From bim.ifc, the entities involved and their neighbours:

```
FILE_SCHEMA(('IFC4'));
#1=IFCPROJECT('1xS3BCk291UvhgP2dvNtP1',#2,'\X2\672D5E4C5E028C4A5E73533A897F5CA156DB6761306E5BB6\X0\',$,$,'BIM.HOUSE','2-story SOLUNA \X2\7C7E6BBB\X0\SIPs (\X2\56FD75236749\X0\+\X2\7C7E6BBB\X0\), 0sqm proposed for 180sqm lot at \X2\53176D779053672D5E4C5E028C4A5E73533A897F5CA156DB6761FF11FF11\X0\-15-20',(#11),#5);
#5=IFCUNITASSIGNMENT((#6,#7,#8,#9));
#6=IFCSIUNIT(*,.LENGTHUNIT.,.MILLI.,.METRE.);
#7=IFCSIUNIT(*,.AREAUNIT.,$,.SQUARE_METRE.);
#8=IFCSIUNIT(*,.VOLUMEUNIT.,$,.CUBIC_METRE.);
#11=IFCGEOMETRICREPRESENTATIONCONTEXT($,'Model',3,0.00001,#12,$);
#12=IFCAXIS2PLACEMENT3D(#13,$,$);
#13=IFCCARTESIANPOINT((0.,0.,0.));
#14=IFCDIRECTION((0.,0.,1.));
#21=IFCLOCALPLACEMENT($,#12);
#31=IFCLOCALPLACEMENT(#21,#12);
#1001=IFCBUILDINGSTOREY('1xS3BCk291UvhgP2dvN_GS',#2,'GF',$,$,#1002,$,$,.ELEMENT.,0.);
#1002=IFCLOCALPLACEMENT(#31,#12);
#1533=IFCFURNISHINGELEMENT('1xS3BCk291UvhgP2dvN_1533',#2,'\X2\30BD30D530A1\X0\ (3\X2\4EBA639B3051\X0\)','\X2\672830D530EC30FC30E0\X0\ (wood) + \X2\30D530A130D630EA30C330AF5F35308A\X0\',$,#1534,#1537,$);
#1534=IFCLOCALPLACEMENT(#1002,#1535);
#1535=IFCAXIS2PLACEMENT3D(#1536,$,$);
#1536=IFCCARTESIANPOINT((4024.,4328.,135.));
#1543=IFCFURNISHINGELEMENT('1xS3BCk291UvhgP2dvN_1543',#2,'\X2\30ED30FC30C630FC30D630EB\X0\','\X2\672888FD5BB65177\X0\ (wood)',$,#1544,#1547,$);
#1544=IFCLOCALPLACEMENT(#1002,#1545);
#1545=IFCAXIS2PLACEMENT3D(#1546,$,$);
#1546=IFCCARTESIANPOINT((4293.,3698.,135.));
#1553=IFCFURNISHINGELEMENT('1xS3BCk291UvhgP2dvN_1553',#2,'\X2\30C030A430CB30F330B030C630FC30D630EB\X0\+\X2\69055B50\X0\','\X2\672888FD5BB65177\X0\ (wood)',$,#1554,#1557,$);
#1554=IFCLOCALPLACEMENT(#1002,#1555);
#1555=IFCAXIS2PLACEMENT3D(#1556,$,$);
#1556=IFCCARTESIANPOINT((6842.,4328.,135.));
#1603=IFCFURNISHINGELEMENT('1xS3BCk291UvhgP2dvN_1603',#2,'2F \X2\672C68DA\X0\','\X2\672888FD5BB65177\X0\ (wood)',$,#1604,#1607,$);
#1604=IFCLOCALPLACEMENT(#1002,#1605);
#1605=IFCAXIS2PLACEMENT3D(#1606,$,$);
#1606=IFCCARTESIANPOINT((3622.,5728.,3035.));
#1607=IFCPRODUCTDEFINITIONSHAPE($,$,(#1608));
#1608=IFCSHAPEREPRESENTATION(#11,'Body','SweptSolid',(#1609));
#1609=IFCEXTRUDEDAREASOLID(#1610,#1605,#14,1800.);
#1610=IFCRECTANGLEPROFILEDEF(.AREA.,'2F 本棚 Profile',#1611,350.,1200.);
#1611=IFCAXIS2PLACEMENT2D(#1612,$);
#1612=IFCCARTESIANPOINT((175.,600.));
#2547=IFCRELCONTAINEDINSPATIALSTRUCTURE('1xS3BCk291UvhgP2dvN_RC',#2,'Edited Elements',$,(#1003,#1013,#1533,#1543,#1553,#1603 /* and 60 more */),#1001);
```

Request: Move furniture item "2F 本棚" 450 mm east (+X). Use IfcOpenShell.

```python
import ifcopenshell
import ifcopenshell.api.geometry
import ifcopenshell.util.placement

model = ifcopenshell.open("bim.ifc")

item = model.by_id(1603)
matrix = ifcopenshell.util.placement.get_local_placement(item.ObjectPlacement)
matrix[0, 3] += 450.0
ifcopenshell.api.geometry.edit_object_placement(model, product=item, matrix=matrix, is_si=False)

print(ifcopenshell.util.placement.get_local_placement(item.ObjectPlacement).round(3) + 0.0)

model.write("bim_edited.ifc")
```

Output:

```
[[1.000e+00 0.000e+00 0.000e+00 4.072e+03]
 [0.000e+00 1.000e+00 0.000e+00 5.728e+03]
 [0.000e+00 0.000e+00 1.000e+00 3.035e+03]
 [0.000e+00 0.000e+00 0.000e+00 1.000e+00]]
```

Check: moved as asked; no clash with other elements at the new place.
